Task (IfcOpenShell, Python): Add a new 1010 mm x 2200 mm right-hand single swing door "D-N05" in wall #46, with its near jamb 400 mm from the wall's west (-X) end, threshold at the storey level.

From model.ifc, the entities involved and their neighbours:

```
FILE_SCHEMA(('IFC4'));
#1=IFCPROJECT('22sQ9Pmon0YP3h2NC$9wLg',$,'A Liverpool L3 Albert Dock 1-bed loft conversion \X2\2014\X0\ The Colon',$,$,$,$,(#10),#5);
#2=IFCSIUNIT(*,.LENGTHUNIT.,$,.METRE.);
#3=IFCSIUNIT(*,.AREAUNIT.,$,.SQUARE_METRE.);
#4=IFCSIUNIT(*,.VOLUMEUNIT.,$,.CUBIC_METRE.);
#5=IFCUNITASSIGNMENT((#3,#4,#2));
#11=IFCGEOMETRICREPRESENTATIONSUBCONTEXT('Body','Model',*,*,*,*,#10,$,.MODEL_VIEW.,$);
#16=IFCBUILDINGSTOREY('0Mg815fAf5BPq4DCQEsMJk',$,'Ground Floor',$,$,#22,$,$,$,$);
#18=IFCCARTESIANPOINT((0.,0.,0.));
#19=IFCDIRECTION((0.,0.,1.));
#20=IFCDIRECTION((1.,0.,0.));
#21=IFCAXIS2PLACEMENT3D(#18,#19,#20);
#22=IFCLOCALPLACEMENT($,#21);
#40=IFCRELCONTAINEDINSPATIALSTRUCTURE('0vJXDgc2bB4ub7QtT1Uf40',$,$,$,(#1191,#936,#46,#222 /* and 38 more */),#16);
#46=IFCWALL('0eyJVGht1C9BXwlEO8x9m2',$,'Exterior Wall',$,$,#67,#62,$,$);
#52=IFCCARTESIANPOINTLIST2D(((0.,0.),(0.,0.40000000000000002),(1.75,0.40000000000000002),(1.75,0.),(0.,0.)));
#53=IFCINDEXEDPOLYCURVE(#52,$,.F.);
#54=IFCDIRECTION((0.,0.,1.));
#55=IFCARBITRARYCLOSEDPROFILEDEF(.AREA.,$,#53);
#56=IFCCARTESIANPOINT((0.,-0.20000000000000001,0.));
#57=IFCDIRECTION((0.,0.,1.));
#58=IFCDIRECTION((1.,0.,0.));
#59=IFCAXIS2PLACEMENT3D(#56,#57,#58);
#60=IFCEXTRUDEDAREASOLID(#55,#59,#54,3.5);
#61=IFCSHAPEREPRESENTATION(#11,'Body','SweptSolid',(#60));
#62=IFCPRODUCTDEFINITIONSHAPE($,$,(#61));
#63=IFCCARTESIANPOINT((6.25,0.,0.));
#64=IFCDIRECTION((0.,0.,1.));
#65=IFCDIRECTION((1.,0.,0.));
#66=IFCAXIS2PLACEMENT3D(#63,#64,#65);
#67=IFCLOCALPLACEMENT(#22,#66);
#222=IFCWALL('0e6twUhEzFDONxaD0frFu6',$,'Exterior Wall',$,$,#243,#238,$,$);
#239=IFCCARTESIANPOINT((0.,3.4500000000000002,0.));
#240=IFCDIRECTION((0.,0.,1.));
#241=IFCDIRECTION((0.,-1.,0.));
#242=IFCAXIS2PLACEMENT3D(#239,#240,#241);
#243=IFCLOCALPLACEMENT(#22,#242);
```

```python
import numpy as np
import ifcopenshell
import ifcopenshell.api.feature
import ifcopenshell.api.geometry
import ifcopenshell.api.root
import ifcopenshell.api.spatial
import ifcopenshell.geom
import ifcopenshell.util.element
import ifcopenshell.util.placement
import ifcopenshell.util.representation
import ifcopenshell.util.shape
import ifcopenshell.util.unit

model = ifcopenshell.open("model.ifc")
unit_scale = ifcopenshell.util.unit.calculate_unit_scale(model)
settings = ifcopenshell.geom.settings()


def volume(element):
    """Net volume in cubic metres, openings subtracted."""
    shape = ifcopenshell.geom.create_shape(settings, element)
    return ifcopenshell.util.shape.get_volume(shape.geometry)


wall = model.by_guid("0eyJVGht1C9BXwlEO8x9m2")
storey = ifcopenshell.util.element.get_container(wall, ifc_class="IfcBuildingStorey")
context = ifcopenshell.util.representation.get_context(model, "Model", "Body", "MODEL_VIEW")
before = volume(wall)

width, height, from_end, sill = 1.01, 2.2, 0.4, 0.0  # metres

# The wall runs along its own X axis, and the end named is its -X end.
wall_shape = ifcopenshell.geom.create_shape(settings, wall)
x, y, z = ifcopenshell.util.shape.get_vertices(wall_shape.geometry).T
start = x.min() + from_end
face, thickness = float(y.min()), float(y.max() - y.min())
wall_matrix = ifcopenshell.util.placement.get_local_placement(wall.ObjectPlacement)
level = ifcopenshell.util.placement.get_local_placement(storey.ObjectPlacement)[2, 3]


def in_wall(x, y):
    """Placement at x, y metres in the wall's axes, at sill height."""
    matrix = wall_matrix.copy()
    matrix[:, 3] = wall_matrix @ np.array([x / unit_scale, y / unit_scale, 0.0, 1.0])
    matrix[2, 3] = level + sill / unit_scale
    return matrix


# Opening: a box that overshoots both wall faces by 50 mm.
opening = ifcopenshell.api.root.create_entity(model, ifc_class="IfcOpeningElement", predefined_type="OPENING")
box = ifcopenshell.api.geometry.add_wall_representation(
    model, context=context, length=width, height=height, thickness=thickness + 0.1
)
ifcopenshell.api.geometry.assign_representation(model, product=opening, representation=box)
ifcopenshell.api.geometry.edit_object_placement(model, product=opening, matrix=in_wall(start, face - 0.05), is_si=False)
ifcopenshell.api.feature.add_feature(model, feature=opening, element=wall)

door = ifcopenshell.api.root.create_entity(model, ifc_class="IfcDoor", name="D-N05", predefined_type="DOOR")
door.OverallWidth, door.OverallHeight = width / unit_scale, height / unit_scale
door.OperationType = "SINGLE_SWING_RIGHT"
body = ifcopenshell.api.geometry.add_door_representation(
    model,
    context=context,
    overall_width=door.OverallWidth,
    overall_height=door.OverallHeight,
    operation_type="SINGLE_SWING_RIGHT",
    lining_properties={"LiningDepth": thickness / unit_scale, "ThresholdDepth": thickness / unit_scale},
)
ifcopenshell.api.geometry.assign_representation(model, product=door, representation=body)
ifcopenshell.api.spatial.assign_container(model, products=[door], relating_structure=storey)
ifcopenshell.api.feature.add_filling(model, opening=opening, element=door)

# The lining spans the wall, so the door starts at the wall face.
ifcopenshell.api.geometry.edit_object_placement(model, product=door, matrix=in_wall(start, face), is_si=False)

after = volume(wall)

print(f"wall volume {before:.3f} -> {after:.3f} m3")

model.write("model_v2.ifc")
```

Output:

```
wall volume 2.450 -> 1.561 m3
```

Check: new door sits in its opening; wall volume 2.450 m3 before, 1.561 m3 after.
